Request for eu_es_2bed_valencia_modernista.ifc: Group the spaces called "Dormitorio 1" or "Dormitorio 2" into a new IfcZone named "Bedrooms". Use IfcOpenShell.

First a look at what the model holds.

```python
import ifcopenshell

model = ifcopenshell.open("eu_es_2bed_valencia_modernista.ifc")
print(model.schema)
seen = {}
for space in model.by_type("IfcSpace"):
    seen[space.LongName] = seen.get(space.LongName, 0) + 1
for name, count in sorted(seen.items(), key=str):
    print(count, "x", name)
print("zones:", [z.Name for z in model.by_type("IfcZone")][:20])
```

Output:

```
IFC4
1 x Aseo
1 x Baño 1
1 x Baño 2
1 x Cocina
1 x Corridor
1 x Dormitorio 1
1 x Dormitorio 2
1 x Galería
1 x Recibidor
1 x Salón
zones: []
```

```python
import ifcopenshell
import ifcopenshell.api.group
import ifcopenshell.api.root

model = ifcopenshell.open("eu_es_2bed_valencia_modernista.ifc")

names = {"Dormitorio 1", "Dormitorio 2"}
spaces = [s for s in model.by_type("IfcSpace") if s.LongName in names]

zone = ifcopenshell.api.root.create_entity(model, ifc_class="IfcZone", name="Bedrooms")
ifcopenshell.api.group.assign_group(model, products=spaces, group=zone)
print(len(spaces), "spaces in", zone.Name)

model.write("eu_es_2bed_valencia_modernista_rev.ifc")
```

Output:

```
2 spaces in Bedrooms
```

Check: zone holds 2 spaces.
